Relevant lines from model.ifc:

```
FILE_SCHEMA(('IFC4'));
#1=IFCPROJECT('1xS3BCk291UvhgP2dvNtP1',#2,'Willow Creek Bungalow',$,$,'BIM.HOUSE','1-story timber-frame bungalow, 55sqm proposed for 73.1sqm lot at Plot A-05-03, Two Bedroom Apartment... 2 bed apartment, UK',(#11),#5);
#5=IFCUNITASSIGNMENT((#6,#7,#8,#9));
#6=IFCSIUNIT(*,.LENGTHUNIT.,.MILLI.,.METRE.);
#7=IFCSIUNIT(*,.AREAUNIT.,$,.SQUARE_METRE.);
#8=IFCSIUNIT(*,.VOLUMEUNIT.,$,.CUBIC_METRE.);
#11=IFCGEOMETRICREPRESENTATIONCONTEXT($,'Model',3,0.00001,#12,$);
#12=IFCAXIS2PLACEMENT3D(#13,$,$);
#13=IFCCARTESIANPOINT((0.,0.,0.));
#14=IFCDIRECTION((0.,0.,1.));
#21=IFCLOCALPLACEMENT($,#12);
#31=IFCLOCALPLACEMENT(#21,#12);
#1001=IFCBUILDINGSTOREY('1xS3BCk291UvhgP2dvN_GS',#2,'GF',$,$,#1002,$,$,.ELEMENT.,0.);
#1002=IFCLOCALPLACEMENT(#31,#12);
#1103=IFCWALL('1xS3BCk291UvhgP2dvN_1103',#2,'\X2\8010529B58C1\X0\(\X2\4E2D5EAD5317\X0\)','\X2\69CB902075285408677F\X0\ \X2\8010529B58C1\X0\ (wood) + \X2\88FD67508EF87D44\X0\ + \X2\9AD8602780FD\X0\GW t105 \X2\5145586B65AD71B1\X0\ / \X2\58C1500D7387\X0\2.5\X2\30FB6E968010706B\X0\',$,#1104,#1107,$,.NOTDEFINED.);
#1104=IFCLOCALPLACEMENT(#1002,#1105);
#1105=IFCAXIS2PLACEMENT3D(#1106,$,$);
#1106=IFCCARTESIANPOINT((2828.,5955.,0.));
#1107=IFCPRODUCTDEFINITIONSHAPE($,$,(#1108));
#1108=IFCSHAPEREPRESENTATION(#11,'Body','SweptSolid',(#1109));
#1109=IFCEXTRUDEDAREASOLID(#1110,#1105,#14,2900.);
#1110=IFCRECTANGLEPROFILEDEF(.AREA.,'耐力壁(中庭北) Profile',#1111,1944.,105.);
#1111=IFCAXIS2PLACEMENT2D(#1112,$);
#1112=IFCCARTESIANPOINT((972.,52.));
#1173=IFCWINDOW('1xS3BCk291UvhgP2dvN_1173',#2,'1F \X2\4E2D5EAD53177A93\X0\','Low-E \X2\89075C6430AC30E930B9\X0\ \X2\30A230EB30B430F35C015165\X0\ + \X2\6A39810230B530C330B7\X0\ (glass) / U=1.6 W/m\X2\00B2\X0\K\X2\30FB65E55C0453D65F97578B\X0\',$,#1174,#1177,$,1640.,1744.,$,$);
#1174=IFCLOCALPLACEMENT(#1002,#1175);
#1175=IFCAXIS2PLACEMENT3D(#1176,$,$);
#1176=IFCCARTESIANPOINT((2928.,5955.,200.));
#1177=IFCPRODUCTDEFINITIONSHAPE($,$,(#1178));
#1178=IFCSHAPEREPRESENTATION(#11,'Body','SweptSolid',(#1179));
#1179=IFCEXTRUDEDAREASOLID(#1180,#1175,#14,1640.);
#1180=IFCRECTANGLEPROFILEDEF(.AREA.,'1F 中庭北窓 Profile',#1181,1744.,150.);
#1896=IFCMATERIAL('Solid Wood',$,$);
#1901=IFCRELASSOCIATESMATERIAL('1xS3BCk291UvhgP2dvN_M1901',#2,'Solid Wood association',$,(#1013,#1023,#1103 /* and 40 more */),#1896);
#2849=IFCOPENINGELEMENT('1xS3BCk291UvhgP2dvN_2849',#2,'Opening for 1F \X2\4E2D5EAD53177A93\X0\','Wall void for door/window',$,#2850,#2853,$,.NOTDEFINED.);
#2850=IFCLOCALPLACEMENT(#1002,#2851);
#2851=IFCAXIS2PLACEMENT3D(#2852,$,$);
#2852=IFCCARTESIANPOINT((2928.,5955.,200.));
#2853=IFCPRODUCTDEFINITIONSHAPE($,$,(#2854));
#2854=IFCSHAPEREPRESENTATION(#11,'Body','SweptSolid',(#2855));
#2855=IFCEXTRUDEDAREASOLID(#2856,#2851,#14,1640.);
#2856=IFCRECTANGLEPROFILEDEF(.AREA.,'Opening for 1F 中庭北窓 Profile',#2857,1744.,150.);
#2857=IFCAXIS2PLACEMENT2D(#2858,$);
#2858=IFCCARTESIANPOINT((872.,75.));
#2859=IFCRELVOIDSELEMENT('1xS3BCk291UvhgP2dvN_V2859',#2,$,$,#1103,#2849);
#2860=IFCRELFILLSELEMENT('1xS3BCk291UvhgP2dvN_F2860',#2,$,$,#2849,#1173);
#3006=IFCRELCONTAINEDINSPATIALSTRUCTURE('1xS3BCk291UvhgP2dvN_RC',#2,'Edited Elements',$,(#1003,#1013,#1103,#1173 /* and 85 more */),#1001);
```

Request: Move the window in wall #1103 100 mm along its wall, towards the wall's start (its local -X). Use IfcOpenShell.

```python
import ifcopenshell
import ifcopenshell.api.geometry
import ifcopenshell.util.placement
import ifcopenshell.util.unit

model = ifcopenshell.open("model.ifc")
unit_scale = ifcopenshell.util.unit.calculate_unit_scale(model)

window = model.by_id(1173)
opening = window.FillsVoids[0].RelatingOpeningElement
wall = opening.VoidsElements[0].RelatingBuildingElement

wall_matrix = ifcopenshell.util.placement.get_local_placement(wall.ObjectPlacement)
shift = wall_matrix[:3, 0] * -0.1 / unit_scale
before = ifcopenshell.util.placement.get_local_placement(window.ObjectPlacement)[:3, 3].copy()

# The window is not placed relative to its opening, so move both.
for product in (opening, window):
    matrix = ifcopenshell.util.placement.get_local_placement(product.ObjectPlacement)
    matrix[:3, 3] += shift
    ifcopenshell.api.geometry.edit_object_placement(model, product=product, matrix=matrix, is_si=False)

after = ifcopenshell.util.placement.get_local_placement(window.ObjectPlacement)[:3, 3]
print("window moved by", (after - before).round(3) + 0.0)

model.write("model_edited.ifc")
```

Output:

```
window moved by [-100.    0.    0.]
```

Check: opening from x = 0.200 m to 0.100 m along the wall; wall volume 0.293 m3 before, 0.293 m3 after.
